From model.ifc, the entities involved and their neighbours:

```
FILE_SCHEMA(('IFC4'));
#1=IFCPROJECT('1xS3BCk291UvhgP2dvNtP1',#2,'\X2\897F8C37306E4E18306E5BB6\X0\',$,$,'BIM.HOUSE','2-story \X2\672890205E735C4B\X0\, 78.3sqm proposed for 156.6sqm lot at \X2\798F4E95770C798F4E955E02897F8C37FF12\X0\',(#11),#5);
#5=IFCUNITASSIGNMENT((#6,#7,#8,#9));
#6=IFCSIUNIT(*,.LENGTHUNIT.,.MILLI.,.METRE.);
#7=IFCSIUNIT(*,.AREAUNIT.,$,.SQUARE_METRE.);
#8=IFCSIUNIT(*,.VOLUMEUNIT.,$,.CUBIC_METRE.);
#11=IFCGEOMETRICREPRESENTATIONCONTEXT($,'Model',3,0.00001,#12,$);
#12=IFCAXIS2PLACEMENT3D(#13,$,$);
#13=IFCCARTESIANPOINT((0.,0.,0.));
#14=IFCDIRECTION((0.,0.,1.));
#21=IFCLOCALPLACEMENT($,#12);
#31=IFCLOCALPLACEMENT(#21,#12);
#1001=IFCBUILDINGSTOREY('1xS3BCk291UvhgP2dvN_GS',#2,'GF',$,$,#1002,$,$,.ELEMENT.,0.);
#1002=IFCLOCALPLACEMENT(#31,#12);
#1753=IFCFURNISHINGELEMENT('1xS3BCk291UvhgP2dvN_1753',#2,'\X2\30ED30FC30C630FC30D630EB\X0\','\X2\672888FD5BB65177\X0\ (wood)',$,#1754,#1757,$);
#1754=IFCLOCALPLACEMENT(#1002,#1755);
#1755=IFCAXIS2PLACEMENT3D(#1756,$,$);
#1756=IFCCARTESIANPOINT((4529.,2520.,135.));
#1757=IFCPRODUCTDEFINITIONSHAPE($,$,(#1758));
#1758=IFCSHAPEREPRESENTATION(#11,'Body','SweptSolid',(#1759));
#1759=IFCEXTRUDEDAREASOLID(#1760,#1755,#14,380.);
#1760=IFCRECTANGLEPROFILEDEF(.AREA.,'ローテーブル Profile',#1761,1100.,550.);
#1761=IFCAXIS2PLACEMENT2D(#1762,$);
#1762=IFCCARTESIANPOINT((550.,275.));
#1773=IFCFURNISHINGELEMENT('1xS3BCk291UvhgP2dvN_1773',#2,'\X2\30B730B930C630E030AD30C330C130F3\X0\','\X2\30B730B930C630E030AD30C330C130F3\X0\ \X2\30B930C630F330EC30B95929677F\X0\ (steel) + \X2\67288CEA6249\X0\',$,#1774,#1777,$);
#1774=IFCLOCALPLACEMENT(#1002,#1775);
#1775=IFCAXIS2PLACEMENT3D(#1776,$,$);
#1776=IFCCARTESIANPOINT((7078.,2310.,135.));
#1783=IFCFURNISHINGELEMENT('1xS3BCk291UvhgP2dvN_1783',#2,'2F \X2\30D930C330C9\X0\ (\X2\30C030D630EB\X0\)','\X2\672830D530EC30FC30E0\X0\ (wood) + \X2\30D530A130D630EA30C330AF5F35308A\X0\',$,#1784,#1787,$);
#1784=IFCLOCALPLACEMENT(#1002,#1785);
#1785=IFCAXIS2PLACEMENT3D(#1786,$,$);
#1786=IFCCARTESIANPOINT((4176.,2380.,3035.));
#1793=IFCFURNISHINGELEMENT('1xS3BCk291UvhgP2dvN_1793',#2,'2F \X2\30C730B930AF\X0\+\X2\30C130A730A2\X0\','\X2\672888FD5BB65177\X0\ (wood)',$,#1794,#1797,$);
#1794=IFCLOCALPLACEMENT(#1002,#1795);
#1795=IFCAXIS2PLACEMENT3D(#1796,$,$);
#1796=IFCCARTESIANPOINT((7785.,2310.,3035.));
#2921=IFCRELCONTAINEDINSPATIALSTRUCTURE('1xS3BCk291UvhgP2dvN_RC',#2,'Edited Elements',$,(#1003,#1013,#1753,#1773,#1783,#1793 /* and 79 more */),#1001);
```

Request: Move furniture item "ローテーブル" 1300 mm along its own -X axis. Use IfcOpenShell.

```python
import ifcopenshell
import ifcopenshell.api.geometry
import ifcopenshell.util.placement

model = ifcopenshell.open("model.ifc")

item = model.by_guid("1xS3BCk291UvhgP2dvN_1753")
matrix = ifcopenshell.util.placement.get_local_placement(item.ObjectPlacement)
matrix[:3, 3] -= matrix[:3, 0] * 1300.0
ifcopenshell.api.geometry.edit_object_placement(model, product=item, matrix=matrix, is_si=False)

print(ifcopenshell.util.placement.get_local_placement(item.ObjectPlacement).round(3) + 0.0)

model.write("model_rev.ifc")
```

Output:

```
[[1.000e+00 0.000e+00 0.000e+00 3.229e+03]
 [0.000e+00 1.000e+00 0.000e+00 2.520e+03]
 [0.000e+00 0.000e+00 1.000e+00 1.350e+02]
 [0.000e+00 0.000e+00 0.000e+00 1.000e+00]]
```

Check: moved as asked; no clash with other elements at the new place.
